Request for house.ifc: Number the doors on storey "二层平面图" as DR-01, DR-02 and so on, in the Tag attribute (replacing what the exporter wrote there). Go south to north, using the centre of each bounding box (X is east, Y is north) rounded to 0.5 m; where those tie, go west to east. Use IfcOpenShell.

First a look at what the model holds.

```python
import ifcopenshell
import ifcopenshell.util.element
import ifcopenshell.util.placement

model = ifcopenshell.open("house.ifc")
print(model.schema)
storey = next(s for s in model.by_type("IfcBuildingStorey") if s.Name == "二层平面图")
doors = [e for e in ifcopenshell.util.element.get_decomposition(storey) if e.is_a("IfcDoor")]
for e in sorted(doors, key=lambda e: e.id()):
    origin = ifcopenshell.util.placement.get_local_placement(e.ObjectPlacement)[:3, 3]
    print(e.id(), e.Tag, e.Name, origin.round(2) + 0.0, sep=" | ")
```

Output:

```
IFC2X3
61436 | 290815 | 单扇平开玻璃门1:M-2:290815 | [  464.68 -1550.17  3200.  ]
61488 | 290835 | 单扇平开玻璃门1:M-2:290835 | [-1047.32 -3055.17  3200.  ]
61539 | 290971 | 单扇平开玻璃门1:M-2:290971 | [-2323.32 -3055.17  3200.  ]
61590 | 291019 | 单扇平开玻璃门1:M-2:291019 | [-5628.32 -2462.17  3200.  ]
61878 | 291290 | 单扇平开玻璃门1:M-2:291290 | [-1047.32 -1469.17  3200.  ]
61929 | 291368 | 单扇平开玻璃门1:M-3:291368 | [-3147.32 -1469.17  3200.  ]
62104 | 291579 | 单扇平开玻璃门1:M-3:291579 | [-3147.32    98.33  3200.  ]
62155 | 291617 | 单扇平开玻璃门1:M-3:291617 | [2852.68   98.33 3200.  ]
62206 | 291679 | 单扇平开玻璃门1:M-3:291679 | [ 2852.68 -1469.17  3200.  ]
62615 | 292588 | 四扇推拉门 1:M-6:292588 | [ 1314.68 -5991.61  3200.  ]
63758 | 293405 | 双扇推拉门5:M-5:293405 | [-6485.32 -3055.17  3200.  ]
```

```python
import ifcopenshell
import ifcopenshell.geom
import ifcopenshell.util.element
import ifcopenshell.util.shape

model = ifcopenshell.open("house.ifc")
settings = ifcopenshell.geom.settings()
settings.set("use-world-coords", True)


def centre(element):
    shape = ifcopenshell.geom.create_shape(settings, element)
    return ifcopenshell.util.shape.get_bbox_centroid(shape.geometry)


storey = next(s for s in model.by_type("IfcBuildingStorey") if s.Name == "二层平面图")
doors = [e for e in ifcopenshell.util.element.get_decomposition(storey) if e.is_a("IfcDoor")]

# Insertion points can sit at a corner or the storey origin, so sort by the geometry (in metres).
centres = {e: centre(e) for e in doors}
doors.sort(key=lambda e: (round(centres[e][1] / 0.5), centres[e][0]))

for i, e in enumerate(doors, start=1):
    number = f"DR-{i:02d}"
    e.Tag = number
    print(e.id(), number)

model.write("house_updated.ifc")
```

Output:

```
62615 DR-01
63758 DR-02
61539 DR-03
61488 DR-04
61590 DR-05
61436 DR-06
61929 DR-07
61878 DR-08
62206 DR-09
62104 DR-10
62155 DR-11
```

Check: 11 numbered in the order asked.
